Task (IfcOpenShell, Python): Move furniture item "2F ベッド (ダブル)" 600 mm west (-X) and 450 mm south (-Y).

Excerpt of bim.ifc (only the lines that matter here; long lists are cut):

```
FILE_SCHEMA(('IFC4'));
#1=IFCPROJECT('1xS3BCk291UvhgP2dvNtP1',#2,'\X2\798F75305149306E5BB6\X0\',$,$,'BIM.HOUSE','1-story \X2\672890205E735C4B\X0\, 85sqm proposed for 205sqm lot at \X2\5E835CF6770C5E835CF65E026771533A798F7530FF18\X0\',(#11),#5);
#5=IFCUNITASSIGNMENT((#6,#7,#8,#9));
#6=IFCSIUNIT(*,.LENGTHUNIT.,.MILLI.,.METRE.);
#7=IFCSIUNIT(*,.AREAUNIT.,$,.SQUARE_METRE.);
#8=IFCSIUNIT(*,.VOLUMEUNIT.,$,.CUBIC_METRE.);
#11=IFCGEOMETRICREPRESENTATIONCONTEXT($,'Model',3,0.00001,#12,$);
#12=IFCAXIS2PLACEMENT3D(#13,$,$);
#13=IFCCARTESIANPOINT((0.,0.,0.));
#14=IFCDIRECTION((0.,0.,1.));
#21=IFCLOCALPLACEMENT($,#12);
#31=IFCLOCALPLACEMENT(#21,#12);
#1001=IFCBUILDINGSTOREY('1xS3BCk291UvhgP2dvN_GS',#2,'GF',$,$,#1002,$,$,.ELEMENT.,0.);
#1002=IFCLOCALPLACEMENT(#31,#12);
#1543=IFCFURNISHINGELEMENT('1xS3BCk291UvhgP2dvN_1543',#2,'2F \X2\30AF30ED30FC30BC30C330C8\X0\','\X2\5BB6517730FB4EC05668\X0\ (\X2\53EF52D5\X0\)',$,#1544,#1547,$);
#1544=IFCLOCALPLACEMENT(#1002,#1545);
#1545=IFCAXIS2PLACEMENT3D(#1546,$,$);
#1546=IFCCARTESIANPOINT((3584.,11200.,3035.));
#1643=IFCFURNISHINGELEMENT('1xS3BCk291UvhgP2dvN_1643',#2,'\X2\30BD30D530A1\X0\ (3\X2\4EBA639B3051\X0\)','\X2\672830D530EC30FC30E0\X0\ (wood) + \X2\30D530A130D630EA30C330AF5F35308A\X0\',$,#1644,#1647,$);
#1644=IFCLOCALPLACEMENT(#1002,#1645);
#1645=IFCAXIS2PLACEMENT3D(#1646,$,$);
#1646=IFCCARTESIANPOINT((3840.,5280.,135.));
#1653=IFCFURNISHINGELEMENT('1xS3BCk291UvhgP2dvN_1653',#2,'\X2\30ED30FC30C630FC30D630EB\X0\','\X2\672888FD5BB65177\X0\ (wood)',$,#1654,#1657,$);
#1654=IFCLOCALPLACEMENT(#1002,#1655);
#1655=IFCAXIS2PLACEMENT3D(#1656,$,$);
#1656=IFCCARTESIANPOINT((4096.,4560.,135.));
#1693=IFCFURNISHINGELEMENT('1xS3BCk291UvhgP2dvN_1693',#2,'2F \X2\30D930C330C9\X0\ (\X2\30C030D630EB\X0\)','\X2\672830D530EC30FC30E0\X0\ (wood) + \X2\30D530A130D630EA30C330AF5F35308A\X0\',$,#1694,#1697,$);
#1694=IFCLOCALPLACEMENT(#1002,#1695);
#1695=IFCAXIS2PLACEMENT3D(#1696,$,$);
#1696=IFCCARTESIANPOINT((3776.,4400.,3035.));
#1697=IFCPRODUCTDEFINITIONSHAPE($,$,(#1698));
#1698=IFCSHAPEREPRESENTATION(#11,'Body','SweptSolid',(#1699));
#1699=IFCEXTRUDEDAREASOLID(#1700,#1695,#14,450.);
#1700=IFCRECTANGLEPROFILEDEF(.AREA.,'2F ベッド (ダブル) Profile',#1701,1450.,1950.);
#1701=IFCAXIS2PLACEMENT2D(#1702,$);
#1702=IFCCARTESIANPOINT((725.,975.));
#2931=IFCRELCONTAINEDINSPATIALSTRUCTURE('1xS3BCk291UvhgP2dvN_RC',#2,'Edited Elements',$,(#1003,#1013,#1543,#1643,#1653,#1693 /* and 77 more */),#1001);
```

```python
import ifcopenshell
import ifcopenshell.api.geometry
import ifcopenshell.util.placement
import ifcopenshell.util.unit

model = ifcopenshell.open("bim.ifc")
unit_scale = ifcopenshell.util.unit.calculate_unit_scale(model)

item = model.by_guid("1xS3BCk291UvhgP2dvN_1693")
matrix = ifcopenshell.util.placement.get_local_placement(item.ObjectPlacement)
matrix[0, 3] -= 0.6 / unit_scale
matrix[1, 3] -= 0.45 / unit_scale
ifcopenshell.api.geometry.edit_object_placement(model, product=item, matrix=matrix, is_si=False)

print(ifcopenshell.util.placement.get_local_placement(item.ObjectPlacement).round(3) + 0.0)

model.write("bim_v2.ifc")
```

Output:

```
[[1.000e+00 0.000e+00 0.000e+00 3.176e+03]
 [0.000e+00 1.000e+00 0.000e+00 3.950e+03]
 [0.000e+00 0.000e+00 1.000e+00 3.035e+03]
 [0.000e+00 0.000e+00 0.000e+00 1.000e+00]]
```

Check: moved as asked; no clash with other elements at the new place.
